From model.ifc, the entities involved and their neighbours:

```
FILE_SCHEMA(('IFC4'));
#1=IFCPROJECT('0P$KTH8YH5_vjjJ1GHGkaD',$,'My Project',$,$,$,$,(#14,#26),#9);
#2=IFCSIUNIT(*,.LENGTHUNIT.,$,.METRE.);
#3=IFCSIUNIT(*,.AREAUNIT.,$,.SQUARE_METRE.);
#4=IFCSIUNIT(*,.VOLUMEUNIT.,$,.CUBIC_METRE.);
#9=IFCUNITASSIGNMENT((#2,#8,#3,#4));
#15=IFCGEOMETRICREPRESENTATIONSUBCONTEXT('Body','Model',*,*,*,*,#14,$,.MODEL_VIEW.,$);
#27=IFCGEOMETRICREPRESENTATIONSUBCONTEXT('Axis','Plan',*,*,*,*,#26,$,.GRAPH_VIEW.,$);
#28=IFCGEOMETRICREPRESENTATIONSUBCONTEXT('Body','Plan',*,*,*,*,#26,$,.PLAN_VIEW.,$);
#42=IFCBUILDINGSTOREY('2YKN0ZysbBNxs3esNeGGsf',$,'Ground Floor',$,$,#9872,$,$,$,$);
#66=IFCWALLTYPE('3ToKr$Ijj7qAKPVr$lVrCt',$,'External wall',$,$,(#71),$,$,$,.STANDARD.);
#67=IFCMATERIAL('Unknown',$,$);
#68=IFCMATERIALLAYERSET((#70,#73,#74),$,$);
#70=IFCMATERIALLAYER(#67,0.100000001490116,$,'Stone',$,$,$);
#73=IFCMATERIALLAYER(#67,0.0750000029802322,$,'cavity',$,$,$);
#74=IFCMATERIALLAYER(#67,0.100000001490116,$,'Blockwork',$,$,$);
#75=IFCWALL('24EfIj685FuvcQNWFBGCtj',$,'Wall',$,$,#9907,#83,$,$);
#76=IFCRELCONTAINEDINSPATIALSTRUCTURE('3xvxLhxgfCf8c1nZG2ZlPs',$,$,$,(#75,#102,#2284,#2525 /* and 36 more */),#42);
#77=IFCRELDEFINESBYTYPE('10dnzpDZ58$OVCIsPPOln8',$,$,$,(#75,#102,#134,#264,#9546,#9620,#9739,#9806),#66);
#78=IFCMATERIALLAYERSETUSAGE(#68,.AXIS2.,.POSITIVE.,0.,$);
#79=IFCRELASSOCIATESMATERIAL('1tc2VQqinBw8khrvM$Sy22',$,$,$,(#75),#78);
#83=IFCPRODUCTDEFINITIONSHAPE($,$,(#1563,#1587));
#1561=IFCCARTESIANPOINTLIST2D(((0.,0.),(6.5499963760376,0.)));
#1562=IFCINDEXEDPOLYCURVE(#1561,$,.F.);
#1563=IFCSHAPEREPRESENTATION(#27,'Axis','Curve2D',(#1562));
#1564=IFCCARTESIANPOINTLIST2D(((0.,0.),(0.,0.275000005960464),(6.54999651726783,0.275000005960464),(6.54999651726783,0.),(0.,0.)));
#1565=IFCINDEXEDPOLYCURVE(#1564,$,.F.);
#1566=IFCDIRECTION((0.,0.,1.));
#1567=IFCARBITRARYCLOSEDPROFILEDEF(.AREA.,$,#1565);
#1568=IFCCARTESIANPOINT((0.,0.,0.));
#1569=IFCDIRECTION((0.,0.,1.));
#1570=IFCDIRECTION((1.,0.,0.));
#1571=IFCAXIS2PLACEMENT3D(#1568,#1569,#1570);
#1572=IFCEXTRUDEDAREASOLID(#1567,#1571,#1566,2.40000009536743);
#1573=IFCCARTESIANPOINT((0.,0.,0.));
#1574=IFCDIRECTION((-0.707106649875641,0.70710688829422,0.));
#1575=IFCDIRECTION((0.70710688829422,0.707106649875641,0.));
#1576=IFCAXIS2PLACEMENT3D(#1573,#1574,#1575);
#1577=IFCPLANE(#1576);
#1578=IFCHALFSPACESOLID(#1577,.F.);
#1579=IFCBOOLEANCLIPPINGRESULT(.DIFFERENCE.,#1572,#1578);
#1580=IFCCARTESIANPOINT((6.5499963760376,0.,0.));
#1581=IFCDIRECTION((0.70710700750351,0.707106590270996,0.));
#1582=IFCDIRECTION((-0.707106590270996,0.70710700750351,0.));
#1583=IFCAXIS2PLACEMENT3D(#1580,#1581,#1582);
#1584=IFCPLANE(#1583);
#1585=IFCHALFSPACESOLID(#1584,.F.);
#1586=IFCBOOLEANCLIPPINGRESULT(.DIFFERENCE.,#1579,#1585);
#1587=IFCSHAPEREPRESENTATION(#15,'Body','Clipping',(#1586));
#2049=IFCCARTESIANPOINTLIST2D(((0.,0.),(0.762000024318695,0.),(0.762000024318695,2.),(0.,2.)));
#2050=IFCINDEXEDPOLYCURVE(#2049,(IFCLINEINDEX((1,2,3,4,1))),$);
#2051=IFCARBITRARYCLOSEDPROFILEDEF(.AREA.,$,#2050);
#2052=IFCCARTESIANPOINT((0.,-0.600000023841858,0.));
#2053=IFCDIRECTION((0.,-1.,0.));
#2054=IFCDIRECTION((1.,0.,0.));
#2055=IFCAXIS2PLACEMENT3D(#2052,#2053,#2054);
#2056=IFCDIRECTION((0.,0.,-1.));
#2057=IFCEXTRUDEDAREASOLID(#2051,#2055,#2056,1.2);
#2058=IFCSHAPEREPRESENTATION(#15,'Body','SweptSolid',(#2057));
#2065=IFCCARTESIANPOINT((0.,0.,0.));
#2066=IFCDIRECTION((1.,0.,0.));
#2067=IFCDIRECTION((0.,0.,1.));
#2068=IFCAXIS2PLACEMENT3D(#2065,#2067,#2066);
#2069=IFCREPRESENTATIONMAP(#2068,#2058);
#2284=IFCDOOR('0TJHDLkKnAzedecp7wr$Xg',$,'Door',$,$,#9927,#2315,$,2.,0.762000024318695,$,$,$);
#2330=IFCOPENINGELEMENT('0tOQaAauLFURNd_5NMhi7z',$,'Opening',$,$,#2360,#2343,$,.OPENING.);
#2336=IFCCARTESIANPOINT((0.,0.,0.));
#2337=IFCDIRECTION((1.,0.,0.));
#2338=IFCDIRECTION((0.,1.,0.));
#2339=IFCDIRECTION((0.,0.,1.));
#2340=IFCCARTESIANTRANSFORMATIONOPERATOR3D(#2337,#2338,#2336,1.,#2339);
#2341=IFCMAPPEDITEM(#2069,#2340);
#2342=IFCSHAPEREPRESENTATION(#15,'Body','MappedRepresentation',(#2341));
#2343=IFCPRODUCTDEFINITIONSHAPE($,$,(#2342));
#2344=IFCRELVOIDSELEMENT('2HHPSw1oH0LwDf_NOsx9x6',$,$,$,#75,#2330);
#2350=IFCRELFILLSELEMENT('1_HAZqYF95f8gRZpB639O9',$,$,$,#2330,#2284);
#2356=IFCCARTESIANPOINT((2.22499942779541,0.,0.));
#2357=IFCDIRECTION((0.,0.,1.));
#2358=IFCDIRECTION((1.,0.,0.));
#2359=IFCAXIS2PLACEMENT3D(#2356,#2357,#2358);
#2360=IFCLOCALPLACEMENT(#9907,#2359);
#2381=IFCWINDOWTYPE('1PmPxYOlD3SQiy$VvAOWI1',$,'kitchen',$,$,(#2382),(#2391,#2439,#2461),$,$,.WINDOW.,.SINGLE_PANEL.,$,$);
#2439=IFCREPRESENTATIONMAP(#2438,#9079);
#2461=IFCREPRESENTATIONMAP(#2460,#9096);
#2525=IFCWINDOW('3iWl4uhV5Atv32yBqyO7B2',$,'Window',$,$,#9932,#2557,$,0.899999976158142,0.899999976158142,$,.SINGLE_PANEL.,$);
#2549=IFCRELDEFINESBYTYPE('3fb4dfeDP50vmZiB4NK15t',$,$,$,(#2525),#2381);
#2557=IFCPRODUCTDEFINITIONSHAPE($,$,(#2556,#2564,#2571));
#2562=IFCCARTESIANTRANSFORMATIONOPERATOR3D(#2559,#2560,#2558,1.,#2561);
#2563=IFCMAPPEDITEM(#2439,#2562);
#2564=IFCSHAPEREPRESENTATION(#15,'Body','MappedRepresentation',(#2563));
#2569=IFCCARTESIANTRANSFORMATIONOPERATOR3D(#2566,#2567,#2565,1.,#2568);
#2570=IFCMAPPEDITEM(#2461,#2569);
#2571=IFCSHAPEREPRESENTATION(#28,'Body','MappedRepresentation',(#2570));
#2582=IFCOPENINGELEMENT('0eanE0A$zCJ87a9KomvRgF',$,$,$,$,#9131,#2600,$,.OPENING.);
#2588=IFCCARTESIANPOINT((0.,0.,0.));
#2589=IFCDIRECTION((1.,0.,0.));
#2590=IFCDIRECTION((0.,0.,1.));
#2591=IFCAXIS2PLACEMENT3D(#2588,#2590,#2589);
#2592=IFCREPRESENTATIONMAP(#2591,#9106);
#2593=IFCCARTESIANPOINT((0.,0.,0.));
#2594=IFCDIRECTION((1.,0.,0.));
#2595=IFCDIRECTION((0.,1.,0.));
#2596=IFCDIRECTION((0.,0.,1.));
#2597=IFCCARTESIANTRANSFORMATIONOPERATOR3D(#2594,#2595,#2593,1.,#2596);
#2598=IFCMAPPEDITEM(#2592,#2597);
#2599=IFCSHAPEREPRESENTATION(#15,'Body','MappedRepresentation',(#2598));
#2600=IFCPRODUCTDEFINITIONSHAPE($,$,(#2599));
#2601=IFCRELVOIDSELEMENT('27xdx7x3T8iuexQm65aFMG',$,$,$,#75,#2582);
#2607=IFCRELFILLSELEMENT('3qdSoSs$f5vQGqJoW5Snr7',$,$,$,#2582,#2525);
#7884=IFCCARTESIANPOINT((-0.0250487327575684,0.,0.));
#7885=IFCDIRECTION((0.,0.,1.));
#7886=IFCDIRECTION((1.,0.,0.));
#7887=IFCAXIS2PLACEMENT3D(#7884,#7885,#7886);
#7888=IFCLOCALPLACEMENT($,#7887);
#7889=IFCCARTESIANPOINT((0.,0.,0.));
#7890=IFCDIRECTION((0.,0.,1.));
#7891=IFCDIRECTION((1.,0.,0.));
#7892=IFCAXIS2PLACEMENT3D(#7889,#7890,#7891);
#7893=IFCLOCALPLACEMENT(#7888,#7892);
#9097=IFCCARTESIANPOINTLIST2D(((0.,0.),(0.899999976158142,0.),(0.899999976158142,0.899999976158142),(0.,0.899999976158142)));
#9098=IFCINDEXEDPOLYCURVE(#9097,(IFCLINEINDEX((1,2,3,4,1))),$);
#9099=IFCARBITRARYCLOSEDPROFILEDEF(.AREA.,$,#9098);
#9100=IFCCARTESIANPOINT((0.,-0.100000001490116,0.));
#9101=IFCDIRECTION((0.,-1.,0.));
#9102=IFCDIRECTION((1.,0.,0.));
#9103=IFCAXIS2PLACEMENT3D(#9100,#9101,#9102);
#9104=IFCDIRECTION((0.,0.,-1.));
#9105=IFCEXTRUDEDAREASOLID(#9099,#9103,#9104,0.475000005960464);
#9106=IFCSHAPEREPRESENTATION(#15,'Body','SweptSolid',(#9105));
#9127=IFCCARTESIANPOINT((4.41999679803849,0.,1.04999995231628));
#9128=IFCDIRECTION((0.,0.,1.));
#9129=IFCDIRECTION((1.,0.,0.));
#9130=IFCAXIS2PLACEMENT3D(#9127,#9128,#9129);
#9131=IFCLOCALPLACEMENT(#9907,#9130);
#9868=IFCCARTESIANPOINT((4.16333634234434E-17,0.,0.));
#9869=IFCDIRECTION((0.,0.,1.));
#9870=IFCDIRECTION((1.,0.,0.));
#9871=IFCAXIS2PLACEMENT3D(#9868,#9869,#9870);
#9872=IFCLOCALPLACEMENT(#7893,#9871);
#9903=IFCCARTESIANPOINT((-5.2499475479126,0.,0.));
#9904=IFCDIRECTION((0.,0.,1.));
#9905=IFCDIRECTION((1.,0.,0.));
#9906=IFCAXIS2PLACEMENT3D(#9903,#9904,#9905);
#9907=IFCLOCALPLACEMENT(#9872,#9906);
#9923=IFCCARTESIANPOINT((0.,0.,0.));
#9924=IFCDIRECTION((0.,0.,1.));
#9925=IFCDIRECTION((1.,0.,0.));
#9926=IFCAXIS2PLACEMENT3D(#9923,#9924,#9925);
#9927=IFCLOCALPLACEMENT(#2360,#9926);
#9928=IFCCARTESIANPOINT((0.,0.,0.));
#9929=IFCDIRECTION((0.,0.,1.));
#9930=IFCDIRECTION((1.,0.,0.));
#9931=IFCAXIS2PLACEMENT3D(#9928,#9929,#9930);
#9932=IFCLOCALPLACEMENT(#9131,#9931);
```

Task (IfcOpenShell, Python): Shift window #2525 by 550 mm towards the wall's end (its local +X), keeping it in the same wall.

```python
import ifcopenshell
import ifcopenshell.api.geometry
import ifcopenshell.util.placement

model = ifcopenshell.open("model.ifc")

window = model.by_id(2525)
opening = window.FillsVoids[0].RelatingOpeningElement
wall = opening.VoidsElements[0].RelatingBuildingElement

wall_matrix = ifcopenshell.util.placement.get_local_placement(wall.ObjectPlacement)
shift = wall_matrix[:3, 0] * 0.55
before = ifcopenshell.util.placement.get_local_placement(window.ObjectPlacement)[:3, 3].copy()

# The window is placed relative to its opening, so it follows when the opening moves.
matrix = ifcopenshell.util.placement.get_local_placement(opening.ObjectPlacement)
matrix[:3, 3] += shift
ifcopenshell.api.geometry.edit_object_placement(
    model, product=opening, matrix=matrix, is_si=False, should_transform_children=True
)

after = ifcopenshell.util.placement.get_local_placement(window.ObjectPlacement)[:3, 3]
print("window moved by", (after - before).round(3) + 0.0)

model.write("model_edited.ifc")
```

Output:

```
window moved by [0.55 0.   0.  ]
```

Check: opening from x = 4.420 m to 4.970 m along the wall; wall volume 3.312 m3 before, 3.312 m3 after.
